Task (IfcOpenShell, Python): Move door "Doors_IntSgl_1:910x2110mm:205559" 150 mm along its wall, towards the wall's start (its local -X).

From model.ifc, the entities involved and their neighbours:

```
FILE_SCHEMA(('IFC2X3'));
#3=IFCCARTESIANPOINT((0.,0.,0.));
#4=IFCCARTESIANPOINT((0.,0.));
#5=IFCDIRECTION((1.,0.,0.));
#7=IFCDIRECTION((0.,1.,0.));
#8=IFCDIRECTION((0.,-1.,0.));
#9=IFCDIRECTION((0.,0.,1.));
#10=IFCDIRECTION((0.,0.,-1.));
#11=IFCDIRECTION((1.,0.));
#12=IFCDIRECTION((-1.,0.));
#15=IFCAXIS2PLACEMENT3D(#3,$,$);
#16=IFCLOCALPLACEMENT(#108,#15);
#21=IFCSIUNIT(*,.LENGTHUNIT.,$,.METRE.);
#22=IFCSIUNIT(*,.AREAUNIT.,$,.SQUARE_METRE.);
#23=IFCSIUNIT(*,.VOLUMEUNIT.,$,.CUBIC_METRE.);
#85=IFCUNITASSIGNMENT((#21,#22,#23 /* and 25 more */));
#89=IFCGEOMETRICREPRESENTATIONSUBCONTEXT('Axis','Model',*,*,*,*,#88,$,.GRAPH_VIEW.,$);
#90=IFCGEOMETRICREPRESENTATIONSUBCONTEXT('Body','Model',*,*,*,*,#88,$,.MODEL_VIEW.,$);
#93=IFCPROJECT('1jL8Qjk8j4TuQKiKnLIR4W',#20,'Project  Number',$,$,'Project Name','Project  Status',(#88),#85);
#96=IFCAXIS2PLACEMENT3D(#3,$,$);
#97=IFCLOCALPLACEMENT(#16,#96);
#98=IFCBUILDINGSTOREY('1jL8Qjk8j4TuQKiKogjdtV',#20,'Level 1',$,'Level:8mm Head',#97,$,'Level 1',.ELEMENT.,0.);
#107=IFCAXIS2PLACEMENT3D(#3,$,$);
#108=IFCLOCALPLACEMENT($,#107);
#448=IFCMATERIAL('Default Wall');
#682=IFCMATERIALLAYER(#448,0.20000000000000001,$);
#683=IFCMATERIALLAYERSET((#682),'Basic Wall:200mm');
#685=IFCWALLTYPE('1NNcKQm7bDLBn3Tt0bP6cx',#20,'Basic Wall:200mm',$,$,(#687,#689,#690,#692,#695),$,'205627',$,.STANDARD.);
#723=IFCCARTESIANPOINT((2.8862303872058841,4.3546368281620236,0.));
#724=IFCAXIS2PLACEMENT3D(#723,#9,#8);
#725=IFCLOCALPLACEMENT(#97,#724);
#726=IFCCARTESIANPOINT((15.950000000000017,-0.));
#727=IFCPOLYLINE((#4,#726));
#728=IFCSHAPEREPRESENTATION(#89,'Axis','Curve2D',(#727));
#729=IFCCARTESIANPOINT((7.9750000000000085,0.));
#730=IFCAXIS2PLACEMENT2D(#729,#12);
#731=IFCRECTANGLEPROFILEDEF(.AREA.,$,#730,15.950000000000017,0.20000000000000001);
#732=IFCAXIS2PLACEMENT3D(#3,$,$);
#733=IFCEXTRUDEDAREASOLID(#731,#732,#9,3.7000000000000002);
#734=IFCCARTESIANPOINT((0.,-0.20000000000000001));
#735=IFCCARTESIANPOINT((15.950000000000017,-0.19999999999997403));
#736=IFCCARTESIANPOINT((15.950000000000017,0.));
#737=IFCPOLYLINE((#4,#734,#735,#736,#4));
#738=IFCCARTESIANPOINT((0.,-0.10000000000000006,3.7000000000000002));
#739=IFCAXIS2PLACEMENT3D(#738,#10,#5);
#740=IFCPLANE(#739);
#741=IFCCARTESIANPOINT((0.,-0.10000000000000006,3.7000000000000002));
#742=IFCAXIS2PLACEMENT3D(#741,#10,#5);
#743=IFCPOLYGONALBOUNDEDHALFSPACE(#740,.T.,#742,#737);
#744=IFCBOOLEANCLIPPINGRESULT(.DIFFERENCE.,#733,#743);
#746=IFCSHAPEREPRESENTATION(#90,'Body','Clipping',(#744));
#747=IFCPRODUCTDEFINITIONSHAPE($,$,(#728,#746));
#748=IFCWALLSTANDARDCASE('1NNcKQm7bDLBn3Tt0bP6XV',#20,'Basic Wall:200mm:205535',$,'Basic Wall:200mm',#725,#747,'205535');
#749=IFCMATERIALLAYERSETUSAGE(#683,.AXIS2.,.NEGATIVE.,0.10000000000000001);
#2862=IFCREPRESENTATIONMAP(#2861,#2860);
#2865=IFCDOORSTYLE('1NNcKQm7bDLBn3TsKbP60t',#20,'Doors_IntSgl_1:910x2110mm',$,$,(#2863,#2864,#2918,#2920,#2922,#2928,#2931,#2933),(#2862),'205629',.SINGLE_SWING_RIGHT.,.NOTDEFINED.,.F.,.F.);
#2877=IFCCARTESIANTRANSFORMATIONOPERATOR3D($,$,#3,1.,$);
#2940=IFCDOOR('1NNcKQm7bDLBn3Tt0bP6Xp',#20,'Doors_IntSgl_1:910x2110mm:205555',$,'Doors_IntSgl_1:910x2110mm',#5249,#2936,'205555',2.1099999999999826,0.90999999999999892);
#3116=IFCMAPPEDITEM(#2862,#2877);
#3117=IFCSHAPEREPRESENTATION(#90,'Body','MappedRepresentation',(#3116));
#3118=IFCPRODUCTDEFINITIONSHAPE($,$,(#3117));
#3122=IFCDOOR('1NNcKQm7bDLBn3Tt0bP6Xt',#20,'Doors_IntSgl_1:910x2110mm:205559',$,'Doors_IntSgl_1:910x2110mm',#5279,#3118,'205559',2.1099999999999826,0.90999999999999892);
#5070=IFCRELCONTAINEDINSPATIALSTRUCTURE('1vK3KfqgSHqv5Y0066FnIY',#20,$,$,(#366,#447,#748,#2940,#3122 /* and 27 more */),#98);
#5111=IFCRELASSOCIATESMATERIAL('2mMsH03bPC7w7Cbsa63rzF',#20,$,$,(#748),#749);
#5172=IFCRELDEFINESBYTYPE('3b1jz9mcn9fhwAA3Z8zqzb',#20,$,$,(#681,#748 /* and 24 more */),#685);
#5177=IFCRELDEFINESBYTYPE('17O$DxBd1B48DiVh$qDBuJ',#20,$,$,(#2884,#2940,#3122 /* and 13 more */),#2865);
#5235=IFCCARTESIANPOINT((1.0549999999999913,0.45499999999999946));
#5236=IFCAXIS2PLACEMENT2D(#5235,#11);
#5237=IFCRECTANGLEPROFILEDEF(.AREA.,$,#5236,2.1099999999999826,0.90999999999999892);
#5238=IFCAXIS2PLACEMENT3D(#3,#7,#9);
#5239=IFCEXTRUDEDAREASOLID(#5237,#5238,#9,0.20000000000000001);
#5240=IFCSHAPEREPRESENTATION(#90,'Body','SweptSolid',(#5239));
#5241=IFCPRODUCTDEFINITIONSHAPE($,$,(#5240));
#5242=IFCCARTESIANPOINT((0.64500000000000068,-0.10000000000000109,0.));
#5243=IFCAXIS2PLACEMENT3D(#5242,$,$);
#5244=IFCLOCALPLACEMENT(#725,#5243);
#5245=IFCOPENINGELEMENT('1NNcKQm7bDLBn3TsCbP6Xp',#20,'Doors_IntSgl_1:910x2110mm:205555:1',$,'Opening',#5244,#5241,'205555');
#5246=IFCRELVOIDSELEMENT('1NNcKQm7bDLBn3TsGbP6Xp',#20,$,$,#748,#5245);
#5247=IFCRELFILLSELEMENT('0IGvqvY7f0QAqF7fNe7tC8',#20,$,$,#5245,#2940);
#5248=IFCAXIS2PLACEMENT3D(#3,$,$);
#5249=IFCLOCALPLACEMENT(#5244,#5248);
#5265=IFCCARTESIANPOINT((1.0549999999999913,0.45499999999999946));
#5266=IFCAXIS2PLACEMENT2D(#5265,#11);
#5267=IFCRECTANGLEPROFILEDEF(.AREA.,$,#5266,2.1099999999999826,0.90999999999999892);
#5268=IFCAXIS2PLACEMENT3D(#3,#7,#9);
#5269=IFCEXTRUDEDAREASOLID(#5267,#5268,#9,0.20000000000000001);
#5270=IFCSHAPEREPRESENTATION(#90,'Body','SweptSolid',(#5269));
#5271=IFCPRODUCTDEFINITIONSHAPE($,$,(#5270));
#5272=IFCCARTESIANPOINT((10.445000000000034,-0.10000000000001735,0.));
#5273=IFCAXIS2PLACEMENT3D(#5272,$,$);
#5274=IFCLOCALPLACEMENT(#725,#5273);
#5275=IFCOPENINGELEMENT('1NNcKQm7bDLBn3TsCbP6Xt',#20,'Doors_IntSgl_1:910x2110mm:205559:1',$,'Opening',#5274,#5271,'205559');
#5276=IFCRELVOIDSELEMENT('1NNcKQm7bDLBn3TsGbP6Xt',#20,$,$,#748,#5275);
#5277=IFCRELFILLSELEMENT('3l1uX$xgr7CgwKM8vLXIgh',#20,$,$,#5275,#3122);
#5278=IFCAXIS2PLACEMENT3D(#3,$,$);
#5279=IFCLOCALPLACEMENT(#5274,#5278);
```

```python
import ifcopenshell
import ifcopenshell.api.geometry
import ifcopenshell.util.placement

model = ifcopenshell.open("model.ifc")

door = model.by_guid("1NNcKQm7bDLBn3Tt0bP6Xt")
opening = door.FillsVoids[0].RelatingOpeningElement
wall = opening.VoidsElements[0].RelatingBuildingElement

wall_matrix = ifcopenshell.util.placement.get_local_placement(wall.ObjectPlacement)
shift = wall_matrix[:3, 0] * -0.15
before = ifcopenshell.util.placement.get_local_placement(door.ObjectPlacement)[:3, 3].copy()

# The door is placed relative to its opening, so it follows when the opening moves.
matrix = ifcopenshell.util.placement.get_local_placement(opening.ObjectPlacement)
matrix[:3, 3] += shift
ifcopenshell.api.geometry.edit_object_placement(
    model, product=opening, matrix=matrix, is_si=False, should_transform_children=True
)

after = ifcopenshell.util.placement.get_local_placement(door.ObjectPlacement)[:3, 3]
print("door moved by", (after - before).round(3) + 0.0)

model.write("model_v2.ifc")
```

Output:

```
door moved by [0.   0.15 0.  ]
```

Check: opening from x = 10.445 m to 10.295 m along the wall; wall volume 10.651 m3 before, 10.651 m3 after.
